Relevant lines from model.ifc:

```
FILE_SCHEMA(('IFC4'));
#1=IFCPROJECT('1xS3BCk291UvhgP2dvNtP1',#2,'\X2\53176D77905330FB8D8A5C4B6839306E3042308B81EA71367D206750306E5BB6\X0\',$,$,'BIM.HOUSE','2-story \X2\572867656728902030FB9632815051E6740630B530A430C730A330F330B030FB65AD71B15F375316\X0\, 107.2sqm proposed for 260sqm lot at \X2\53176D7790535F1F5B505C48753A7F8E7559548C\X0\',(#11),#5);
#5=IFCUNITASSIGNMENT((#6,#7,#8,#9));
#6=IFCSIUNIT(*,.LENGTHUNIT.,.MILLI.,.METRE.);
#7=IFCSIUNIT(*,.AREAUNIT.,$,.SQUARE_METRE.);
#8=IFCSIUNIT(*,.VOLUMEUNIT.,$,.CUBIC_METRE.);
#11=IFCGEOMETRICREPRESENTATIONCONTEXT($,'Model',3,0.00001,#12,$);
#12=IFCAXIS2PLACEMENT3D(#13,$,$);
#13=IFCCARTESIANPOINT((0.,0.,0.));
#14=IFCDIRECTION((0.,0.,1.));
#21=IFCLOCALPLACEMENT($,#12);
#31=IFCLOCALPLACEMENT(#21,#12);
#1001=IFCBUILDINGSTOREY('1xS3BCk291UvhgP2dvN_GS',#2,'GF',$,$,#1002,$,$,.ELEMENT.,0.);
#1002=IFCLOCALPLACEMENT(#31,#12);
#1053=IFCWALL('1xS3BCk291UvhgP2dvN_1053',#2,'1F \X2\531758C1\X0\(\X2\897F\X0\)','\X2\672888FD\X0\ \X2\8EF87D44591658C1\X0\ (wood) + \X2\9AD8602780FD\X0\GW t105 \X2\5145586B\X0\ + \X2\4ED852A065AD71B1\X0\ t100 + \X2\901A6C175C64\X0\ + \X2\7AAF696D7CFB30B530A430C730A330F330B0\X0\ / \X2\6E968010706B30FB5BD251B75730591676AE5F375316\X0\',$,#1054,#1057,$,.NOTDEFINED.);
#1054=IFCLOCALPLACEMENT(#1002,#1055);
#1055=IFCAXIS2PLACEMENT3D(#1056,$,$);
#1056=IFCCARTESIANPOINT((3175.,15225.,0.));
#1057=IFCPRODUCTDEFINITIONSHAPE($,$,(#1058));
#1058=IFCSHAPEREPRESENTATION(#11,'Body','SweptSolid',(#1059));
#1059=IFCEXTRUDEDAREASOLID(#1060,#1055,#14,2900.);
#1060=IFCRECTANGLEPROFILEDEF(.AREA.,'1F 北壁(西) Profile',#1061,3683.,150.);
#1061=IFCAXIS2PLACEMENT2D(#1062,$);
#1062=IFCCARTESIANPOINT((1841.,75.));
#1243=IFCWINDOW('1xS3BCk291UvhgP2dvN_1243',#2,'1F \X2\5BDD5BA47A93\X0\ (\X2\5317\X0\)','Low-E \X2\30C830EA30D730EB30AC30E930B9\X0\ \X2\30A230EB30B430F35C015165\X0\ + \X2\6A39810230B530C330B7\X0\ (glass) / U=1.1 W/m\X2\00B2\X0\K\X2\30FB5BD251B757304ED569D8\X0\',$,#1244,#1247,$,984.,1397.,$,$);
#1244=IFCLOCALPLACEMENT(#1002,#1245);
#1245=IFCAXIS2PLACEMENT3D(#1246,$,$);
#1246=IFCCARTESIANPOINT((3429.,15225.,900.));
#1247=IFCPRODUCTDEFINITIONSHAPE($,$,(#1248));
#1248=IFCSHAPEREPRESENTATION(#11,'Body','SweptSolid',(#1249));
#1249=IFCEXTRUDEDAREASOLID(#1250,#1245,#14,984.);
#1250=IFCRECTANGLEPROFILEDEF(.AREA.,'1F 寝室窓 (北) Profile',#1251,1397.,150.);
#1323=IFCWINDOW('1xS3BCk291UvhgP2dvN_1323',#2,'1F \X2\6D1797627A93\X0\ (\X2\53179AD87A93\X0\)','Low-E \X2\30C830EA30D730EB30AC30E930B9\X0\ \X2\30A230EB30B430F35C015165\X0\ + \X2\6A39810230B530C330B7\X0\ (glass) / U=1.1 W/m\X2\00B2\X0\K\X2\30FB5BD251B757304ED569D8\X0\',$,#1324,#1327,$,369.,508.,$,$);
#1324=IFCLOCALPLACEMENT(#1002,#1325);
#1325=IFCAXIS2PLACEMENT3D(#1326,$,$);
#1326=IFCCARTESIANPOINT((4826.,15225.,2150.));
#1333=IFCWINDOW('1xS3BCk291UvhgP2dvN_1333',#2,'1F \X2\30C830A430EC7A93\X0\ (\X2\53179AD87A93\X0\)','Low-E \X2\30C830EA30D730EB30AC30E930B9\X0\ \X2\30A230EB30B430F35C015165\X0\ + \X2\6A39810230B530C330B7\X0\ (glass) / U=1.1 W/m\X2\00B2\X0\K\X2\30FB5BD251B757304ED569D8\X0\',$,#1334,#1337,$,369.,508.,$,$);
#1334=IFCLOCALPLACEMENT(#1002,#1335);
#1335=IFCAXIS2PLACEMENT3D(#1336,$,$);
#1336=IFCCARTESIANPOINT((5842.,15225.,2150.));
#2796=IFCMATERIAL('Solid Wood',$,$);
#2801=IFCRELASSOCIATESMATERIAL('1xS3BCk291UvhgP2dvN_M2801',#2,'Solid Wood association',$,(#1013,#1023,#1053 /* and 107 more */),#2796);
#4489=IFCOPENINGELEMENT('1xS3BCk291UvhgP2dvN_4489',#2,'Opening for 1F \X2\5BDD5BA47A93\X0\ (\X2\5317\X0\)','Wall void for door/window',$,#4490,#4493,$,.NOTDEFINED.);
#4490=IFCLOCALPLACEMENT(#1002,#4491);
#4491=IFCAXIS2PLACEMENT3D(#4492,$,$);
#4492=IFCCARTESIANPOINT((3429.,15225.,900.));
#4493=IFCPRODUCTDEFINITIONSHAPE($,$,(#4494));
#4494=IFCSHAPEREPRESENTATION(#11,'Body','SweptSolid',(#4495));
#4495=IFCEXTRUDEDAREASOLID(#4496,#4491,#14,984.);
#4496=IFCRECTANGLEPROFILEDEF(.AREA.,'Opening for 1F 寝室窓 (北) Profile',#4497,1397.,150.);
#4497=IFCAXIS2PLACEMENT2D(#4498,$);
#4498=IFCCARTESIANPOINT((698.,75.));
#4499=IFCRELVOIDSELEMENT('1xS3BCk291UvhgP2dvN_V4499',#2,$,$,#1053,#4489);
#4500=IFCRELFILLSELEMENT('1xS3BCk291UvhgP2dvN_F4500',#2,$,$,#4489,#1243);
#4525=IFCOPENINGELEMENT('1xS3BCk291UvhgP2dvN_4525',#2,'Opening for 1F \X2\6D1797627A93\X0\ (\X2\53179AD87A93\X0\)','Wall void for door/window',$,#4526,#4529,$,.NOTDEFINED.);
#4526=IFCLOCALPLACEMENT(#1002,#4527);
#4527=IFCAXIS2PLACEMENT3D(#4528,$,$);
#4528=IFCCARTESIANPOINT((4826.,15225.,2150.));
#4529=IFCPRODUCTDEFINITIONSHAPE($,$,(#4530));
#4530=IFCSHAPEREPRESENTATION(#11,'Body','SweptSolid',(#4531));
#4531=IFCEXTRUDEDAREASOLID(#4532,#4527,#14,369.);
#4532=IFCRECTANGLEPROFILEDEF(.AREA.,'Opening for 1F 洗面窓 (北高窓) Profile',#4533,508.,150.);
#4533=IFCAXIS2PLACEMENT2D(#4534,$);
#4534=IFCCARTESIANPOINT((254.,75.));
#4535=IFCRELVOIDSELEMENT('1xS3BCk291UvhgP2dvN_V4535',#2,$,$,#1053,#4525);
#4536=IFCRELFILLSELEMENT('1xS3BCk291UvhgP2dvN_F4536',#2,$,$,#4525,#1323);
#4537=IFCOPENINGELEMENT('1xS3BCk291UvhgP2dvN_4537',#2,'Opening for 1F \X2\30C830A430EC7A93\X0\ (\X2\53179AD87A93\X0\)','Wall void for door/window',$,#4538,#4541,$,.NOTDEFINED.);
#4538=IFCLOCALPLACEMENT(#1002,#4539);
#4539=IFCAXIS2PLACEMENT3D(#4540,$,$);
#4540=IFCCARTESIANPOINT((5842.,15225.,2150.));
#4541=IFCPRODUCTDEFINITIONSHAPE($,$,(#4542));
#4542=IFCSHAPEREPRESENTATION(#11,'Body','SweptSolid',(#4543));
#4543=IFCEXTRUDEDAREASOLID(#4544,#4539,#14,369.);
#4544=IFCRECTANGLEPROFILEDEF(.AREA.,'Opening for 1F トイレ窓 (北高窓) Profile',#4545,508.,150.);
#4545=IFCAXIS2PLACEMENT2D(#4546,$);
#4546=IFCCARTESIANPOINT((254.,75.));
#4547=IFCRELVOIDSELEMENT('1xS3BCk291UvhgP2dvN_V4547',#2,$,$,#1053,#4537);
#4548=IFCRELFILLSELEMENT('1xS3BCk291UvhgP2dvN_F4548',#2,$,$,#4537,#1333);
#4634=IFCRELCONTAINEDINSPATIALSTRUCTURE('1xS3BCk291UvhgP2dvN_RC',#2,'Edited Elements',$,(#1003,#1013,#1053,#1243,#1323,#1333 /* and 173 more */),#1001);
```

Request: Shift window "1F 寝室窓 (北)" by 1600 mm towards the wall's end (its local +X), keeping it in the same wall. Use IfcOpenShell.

```python
import ifcopenshell
import ifcopenshell.api.geometry
import ifcopenshell.util.placement

model = ifcopenshell.open("model.ifc")

window = model.by_guid("1xS3BCk291UvhgP2dvN_1243")
opening = window.FillsVoids[0].RelatingOpeningElement
wall = opening.VoidsElements[0].RelatingBuildingElement

wall_matrix = ifcopenshell.util.placement.get_local_placement(wall.ObjectPlacement)
shift = wall_matrix[:3, 0] * 1600.0
before = ifcopenshell.util.placement.get_local_placement(window.ObjectPlacement)[:3, 3].copy()

# The window is not placed relative to its opening, so move both.
for product in (opening, window):
    matrix = ifcopenshell.util.placement.get_local_placement(product.ObjectPlacement)
    matrix[:3, 3] += shift
    ifcopenshell.api.geometry.edit_object_placement(model, product=product, matrix=matrix, is_si=False)

after = ifcopenshell.util.placement.get_local_placement(window.ObjectPlacement)[:3, 3]
print("window moved by", (after - before).round(3) + 0.0)

model.write("model_updated.ifc")
```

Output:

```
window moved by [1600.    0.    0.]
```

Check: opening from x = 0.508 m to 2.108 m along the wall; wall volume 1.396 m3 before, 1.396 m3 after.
